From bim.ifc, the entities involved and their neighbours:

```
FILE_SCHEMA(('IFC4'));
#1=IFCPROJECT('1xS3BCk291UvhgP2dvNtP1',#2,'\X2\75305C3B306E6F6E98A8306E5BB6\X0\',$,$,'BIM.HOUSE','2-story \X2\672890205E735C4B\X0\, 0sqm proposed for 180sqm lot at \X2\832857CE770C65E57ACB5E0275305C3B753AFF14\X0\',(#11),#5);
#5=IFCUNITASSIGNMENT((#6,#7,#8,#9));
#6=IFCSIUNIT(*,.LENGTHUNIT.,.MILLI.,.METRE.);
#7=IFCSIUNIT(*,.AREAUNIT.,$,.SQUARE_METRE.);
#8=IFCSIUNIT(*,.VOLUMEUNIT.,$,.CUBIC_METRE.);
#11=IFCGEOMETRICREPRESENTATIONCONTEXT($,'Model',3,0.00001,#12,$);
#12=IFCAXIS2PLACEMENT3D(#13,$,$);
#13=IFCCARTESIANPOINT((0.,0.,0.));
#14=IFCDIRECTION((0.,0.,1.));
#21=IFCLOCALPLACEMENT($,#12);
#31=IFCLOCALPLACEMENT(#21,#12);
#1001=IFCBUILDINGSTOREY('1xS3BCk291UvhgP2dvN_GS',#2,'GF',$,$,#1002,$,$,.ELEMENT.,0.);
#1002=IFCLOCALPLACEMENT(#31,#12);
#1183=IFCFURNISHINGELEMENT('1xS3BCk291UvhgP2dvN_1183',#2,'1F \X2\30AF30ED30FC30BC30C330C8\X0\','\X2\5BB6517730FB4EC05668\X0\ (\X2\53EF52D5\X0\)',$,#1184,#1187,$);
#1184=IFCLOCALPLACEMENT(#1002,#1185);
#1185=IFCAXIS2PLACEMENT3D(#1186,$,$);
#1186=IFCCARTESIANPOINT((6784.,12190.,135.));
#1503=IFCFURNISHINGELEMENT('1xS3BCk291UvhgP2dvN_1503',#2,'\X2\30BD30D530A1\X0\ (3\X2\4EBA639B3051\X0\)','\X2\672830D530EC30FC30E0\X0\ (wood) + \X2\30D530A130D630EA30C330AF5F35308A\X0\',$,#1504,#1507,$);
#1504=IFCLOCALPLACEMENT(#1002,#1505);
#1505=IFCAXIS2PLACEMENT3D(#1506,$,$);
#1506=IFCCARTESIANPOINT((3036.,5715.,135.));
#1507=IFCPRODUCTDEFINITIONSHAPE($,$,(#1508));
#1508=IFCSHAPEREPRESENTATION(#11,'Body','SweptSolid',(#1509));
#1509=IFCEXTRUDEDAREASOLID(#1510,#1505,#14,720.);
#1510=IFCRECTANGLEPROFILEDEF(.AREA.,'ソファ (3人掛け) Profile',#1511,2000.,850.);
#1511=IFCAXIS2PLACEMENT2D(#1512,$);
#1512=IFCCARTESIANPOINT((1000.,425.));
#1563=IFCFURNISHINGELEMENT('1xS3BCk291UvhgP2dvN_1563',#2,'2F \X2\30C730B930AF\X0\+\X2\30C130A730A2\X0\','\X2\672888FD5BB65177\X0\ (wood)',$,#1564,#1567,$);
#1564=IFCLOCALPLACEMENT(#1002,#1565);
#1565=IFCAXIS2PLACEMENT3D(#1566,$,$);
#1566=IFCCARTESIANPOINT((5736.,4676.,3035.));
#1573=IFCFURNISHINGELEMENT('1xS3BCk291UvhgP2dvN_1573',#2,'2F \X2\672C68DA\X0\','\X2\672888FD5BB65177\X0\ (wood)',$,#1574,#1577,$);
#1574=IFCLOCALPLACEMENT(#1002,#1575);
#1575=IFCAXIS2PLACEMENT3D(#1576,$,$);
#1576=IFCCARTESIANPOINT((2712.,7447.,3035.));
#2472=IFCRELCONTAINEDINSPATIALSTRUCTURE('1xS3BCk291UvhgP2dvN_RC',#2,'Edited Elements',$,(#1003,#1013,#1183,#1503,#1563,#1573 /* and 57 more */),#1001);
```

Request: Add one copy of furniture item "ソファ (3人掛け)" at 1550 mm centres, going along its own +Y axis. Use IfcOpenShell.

```python
import ifcopenshell
import ifcopenshell.api.geometry
import ifcopenshell.api.root
import ifcopenshell.util.element
import ifcopenshell.util.placement
import ifcopenshell.util.unit

model = ifcopenshell.open("bim.ifc")
unit_scale = ifcopenshell.util.unit.calculate_unit_scale(model)


def reuse_history(source, copy):
    """copy_class also copies each property set's owner history, people and application; keep the originals."""
    for rel in copy.IsDefinedBy:
        if rel.is_a("IfcRelDefinesByProperties") and (history := rel.RelatingPropertyDefinition.OwnerHistory):
            rel.RelatingPropertyDefinition.OwnerHistory = source.OwnerHistory
            ifcopenshell.util.element.remove_deep2(model, history)


source = model.by_id(1503)
base = ifcopenshell.util.placement.get_local_placement(source.ObjectPlacement)
step = base[:3, 1] * 1.55 / unit_scale

for i in range(1, 2):
    copy = ifcopenshell.api.root.copy_class(model, product=source)
    copy.Representation = ifcopenshell.util.element.copy_deep(
        model, source.Representation, exclude=["IfcGeometricRepresentationContext", "IfcRepresentationMap"]
    )
    reuse_history(source, copy)
    matrix = base.copy()
    matrix[:3, 3] += i * step
    print("added at", matrix[:3, 3].round(3) + 0.0)
    ifcopenshell.api.geometry.edit_object_placement(model, product=copy, matrix=matrix, is_si=False)

model.write("bim_v2.ifc")
```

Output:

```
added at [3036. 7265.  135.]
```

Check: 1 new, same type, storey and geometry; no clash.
